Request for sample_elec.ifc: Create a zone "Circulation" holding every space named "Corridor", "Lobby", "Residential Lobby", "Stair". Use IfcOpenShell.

First a look at what the model holds.

```python
import ifcopenshell

model = ifcopenshell.open("sample_elec.ifc")
print(model.schema)
seen = {}
for space in model.by_type("IfcSpace"):
    seen[space.LongName] = seen.get(space.LongName, 0) + 1
for name, count in sorted(seen.items(), key=str):
    print(count, "x", name)
print("zones:", [z.Name for z in model.by_type("IfcZone")][:20])
```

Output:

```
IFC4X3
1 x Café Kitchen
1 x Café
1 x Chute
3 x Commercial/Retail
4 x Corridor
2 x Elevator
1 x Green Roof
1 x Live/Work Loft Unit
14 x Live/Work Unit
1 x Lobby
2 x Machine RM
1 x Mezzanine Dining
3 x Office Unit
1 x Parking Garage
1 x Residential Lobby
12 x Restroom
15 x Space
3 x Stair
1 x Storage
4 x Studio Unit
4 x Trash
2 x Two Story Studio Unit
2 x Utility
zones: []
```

```python
import ifcopenshell
import ifcopenshell.api.group
import ifcopenshell.api.root

model = ifcopenshell.open("sample_elec.ifc")

names = {"Corridor", "Lobby", "Residential Lobby", "Stair"}
spaces = [s for s in model.by_type("IfcSpace") if s.LongName in names]

zone = ifcopenshell.api.root.create_entity(model, ifc_class="IfcZone", name="Circulation")
ifcopenshell.api.group.assign_group(model, products=spaces, group=zone)
print(len(spaces), "spaces in", zone.Name)

model.write("sample_elec_v2.ifc")
```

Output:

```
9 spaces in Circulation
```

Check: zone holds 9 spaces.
